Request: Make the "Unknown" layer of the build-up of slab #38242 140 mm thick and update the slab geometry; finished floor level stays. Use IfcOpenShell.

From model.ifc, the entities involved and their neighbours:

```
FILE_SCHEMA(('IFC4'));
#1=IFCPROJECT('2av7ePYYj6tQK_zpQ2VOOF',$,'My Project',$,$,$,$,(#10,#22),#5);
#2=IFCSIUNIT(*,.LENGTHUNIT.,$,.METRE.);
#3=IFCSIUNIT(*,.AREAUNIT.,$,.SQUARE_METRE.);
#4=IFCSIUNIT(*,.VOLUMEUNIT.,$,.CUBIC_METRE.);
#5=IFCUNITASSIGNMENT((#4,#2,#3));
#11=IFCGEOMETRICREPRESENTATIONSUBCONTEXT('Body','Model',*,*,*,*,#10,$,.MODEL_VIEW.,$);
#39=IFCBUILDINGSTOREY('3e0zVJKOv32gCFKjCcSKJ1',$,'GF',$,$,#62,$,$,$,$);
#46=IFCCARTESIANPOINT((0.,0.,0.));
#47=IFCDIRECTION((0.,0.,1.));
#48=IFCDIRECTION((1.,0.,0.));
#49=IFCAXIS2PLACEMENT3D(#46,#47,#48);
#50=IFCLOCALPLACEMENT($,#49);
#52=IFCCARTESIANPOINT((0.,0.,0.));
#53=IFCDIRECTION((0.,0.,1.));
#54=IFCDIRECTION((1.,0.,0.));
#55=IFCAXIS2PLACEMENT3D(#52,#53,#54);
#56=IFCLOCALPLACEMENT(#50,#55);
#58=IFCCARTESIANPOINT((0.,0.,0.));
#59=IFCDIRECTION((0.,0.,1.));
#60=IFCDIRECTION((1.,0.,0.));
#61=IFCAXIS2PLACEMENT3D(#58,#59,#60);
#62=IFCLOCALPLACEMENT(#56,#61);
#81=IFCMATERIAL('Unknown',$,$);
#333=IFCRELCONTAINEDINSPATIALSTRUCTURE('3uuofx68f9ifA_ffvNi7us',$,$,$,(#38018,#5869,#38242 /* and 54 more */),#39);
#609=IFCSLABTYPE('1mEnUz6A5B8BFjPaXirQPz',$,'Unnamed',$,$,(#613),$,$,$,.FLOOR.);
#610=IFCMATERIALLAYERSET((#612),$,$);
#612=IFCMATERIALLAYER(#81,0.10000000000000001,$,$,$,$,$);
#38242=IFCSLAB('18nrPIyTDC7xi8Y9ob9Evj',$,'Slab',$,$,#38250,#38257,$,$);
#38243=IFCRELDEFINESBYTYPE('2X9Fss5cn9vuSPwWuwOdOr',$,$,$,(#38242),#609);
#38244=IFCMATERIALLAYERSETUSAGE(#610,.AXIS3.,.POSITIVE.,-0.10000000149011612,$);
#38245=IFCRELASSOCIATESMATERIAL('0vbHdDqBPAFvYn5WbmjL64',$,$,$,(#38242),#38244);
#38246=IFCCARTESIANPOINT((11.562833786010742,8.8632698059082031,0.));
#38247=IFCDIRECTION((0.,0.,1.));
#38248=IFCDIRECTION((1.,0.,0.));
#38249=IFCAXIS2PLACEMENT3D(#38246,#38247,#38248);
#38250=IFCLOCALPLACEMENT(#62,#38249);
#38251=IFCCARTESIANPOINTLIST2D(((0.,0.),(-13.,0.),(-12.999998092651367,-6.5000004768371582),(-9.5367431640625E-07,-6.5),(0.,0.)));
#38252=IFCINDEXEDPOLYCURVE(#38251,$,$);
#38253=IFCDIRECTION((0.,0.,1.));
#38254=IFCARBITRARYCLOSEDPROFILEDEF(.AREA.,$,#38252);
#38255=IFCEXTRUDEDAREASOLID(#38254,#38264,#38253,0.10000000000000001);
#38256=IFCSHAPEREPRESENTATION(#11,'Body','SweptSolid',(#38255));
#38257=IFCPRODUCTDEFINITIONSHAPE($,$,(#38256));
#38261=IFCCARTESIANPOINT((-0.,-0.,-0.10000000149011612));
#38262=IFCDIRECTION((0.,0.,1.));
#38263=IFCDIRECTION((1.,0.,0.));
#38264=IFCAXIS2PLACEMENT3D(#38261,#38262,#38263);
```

```python
import ifcopenshell
import ifcopenshell.util.element
import ifcopenshell.util.representation

model = ifcopenshell.open("model.ifc")

layer_set = model.by_id(610)
layer = next(l for l in layer_set.MaterialLayers if l.Material and l.Material.Name == "Unknown")
change = 0.14 - layer.LayerThickness
layer.LayerThickness += change

# Geometry does not follow the layer set by itself.
slabs = [e for e in ifcopenshell.util.element.get_elements_by_material(model, layer_set) if e.is_a("IfcSlab")]
for slab in sorted(slabs, key=lambda e: e.id()):
    body = ifcopenshell.util.representation.get_representation(slab, "Model", "Body")
    solid = body.Items[0]
    old_depth = solid.Depth
    solid.Depth += change
    # Extruded upwards: lower the start of the extrusion so the top stays.
    x, y, z = solid.Position.Location.Coordinates
    solid.Position.Location = model.createIfcCartesianPoint((x, y, z - change))
    print(slab.id(), f"{old_depth:g} -> {solid.Depth:g}")

# The layers are counted up from the underside, which has moved.
for usage in {ifcopenshell.util.element.get_material(slab) for slab in slabs}:
    usage.OffsetFromReferenceLine -= change

model.write("model_rev.ifc")
```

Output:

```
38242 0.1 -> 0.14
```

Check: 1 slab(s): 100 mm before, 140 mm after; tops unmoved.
